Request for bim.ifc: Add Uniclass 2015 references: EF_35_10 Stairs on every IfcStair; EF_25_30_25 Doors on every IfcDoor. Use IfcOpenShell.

First a look at what the model holds.

```python
import ifcopenshell

model = ifcopenshell.open("bim.ifc")
print(model.schema)
print("classifications:", [c.Name for c in model.by_type("IfcClassification")])
for ifc_class in ("IfcDoor", "IfcRoof", "IfcStair", "IfcWall", "IfcWindow"):
    print(ifc_class, len(model.by_type(ifc_class)))
```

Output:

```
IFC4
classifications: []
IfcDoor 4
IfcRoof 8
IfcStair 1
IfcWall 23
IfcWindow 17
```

```python
import ifcopenshell
import ifcopenshell.api.classification

model = ifcopenshell.open("bim.ifc")

system = ifcopenshell.api.classification.add_classification(model, classification="Uniclass 2015")

codes = {
    "IfcStair": ("EF_35_10", "Stairs"),
    "IfcDoor": ("EF_25_30_25", "Doors"),
}
for ifc_class, (code, name) in codes.items():
    products = model.by_type(ifc_class)
    ifcopenshell.api.classification.add_reference(
        model, products=products, classification=system, identification=code, name=name
    )
    print(code, len(products))

model.write("bim_v2.ifc")
```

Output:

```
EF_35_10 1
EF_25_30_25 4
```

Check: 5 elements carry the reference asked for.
